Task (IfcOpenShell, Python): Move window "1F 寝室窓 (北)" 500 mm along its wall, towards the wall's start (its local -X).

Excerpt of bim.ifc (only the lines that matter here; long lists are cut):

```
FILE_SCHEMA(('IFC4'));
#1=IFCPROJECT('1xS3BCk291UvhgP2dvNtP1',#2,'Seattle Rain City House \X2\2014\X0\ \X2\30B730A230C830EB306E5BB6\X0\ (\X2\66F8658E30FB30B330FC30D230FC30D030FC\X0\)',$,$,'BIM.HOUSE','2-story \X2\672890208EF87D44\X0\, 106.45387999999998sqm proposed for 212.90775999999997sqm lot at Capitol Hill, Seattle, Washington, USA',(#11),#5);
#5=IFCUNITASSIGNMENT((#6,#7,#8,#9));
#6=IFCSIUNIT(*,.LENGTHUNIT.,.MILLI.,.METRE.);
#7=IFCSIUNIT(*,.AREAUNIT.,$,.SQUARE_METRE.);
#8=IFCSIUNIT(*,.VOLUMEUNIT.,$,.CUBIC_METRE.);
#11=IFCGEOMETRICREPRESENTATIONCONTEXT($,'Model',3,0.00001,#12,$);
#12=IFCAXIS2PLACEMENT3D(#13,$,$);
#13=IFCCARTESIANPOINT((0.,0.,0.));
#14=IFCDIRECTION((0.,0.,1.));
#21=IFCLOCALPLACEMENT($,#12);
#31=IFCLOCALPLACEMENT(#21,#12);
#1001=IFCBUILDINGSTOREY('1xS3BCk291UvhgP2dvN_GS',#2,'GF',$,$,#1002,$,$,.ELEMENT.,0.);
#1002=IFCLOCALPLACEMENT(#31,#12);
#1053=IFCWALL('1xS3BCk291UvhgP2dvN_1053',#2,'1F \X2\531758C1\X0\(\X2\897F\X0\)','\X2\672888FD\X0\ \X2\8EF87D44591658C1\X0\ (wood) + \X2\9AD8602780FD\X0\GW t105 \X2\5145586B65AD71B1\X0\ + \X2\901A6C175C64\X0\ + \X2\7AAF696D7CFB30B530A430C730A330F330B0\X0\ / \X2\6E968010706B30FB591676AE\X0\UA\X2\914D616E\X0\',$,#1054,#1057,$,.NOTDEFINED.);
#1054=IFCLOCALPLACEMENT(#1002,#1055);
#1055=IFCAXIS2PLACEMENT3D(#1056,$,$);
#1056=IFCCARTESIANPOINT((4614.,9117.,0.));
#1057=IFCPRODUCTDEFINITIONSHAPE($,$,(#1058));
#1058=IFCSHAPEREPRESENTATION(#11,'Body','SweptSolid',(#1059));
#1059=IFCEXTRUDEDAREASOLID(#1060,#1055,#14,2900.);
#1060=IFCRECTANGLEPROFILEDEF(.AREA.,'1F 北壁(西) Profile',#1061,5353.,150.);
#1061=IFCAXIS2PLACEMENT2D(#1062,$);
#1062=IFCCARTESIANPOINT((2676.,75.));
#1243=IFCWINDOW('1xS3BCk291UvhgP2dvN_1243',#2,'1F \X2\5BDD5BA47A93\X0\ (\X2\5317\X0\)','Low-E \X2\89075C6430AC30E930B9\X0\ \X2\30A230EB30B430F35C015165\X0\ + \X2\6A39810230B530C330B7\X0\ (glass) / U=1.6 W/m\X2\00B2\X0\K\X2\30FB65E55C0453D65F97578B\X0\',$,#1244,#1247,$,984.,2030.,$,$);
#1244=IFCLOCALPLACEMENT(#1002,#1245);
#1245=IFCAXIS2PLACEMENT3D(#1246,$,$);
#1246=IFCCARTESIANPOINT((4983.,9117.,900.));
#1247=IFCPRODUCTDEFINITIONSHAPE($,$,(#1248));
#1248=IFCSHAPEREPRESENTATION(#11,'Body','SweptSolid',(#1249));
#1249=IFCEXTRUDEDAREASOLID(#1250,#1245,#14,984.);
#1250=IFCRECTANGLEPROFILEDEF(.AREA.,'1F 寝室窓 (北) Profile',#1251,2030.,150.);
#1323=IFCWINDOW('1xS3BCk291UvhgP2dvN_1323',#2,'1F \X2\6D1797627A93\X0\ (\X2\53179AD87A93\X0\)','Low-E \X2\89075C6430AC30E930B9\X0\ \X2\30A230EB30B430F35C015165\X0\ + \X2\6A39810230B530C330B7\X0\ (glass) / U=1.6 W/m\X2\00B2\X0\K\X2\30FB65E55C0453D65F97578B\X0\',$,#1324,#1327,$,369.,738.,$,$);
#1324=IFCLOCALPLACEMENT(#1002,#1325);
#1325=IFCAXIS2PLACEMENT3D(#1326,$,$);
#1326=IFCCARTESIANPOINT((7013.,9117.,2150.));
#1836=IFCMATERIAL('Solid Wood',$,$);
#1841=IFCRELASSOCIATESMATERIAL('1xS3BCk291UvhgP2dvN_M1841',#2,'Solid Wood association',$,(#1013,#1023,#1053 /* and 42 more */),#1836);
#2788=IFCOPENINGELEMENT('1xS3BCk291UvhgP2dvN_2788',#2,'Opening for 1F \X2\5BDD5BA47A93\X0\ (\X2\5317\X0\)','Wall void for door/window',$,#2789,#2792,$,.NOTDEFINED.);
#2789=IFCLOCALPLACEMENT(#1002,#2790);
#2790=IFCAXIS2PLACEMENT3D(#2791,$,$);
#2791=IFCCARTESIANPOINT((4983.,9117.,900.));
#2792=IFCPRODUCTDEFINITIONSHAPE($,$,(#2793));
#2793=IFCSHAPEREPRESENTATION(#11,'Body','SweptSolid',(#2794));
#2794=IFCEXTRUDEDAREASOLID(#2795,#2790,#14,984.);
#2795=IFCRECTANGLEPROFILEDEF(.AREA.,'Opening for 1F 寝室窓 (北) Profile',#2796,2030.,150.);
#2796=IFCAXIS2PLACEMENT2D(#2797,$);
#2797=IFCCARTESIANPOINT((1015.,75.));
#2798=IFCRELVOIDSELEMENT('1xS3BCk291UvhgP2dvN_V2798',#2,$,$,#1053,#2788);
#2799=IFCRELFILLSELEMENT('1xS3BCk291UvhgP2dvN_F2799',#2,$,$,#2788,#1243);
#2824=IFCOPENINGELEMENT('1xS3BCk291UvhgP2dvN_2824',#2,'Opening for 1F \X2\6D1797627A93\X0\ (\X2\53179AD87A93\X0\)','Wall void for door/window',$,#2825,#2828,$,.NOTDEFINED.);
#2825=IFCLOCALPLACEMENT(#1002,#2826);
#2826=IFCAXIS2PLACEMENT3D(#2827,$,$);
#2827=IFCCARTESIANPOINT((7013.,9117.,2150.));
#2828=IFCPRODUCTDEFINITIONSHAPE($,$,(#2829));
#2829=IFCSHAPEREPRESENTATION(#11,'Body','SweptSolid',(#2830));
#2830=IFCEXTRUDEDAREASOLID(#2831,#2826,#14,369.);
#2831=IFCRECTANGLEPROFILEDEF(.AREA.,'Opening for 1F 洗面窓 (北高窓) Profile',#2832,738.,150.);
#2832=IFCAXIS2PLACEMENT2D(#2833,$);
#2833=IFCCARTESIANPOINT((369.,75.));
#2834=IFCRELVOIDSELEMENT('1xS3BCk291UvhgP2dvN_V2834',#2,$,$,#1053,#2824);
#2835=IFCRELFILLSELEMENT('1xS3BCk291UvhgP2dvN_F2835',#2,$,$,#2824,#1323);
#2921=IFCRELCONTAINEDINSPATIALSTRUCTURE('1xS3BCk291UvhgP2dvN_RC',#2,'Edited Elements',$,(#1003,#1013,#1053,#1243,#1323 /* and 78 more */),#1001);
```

```python
import ifcopenshell
import ifcopenshell.api.geometry
import ifcopenshell.util.placement

model = ifcopenshell.open("bim.ifc")

window = model.by_id(1243)
opening = window.FillsVoids[0].RelatingOpeningElement
wall = opening.VoidsElements[0].RelatingBuildingElement

wall_matrix = ifcopenshell.util.placement.get_local_placement(wall.ObjectPlacement)
shift = wall_matrix[:3, 0] * -500.0
before = ifcopenshell.util.placement.get_local_placement(window.ObjectPlacement)[:3, 3].copy()

# The window is not placed relative to its opening, so move both.
for product in (opening, window):
    matrix = ifcopenshell.util.placement.get_local_placement(product.ObjectPlacement)
    matrix[:3, 3] += shift
    ifcopenshell.api.geometry.edit_object_placement(model, product=product, matrix=matrix, is_si=False)

after = ifcopenshell.util.placement.get_local_placement(window.ObjectPlacement)[:3, 3]
print("window moved by", (after - before).round(3) + 0.0)

model.write("bim_rev.ifc")
```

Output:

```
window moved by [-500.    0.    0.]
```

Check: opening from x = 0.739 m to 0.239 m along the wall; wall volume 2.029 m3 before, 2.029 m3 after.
